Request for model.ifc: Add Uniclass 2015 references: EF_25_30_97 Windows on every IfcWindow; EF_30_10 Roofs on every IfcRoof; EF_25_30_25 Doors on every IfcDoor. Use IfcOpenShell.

First a look at what the model holds.

```python
import ifcopenshell

model = ifcopenshell.open("model.ifc")
print(model.schema)
print("classifications:", [c.Name for c in model.by_type("IfcClassification")])
for ifc_class in ("IfcDoor", "IfcRoof", "IfcStair", "IfcWall", "IfcWindow"):
    print(ifc_class, len(model.by_type(ifc_class)))
```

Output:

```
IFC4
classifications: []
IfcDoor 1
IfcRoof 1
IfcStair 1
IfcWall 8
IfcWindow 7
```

```python
import ifcopenshell
import ifcopenshell.api.classification

model = ifcopenshell.open("model.ifc")

system = ifcopenshell.api.classification.add_classification(model, classification="Uniclass 2015")

codes = {
    "IfcWindow": ("EF_25_30_97", "Windows"),
    "IfcRoof": ("EF_30_10", "Roofs"),
    "IfcDoor": ("EF_25_30_25", "Doors"),
}
for ifc_class, (code, name) in codes.items():
    products = model.by_type(ifc_class)
    ifcopenshell.api.classification.add_reference(
        model, products=products, classification=system, identification=code, name=name
    )
    print(code, len(products))

model.write("model_rev.ifc")
```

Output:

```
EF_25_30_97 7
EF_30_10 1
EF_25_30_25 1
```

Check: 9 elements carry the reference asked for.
